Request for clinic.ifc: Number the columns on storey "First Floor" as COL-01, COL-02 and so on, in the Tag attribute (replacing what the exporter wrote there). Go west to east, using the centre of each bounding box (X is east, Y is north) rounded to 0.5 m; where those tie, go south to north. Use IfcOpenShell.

First a look at what the model holds.

```python
import ifcopenshell
import ifcopenshell.util.element
import ifcopenshell.util.placement

model = ifcopenshell.open("clinic.ifc")
print(model.schema)
storey = next(s for s in model.by_type("IfcBuildingStorey") if s.Name == "First Floor")
columns = [e for e in ifcopenshell.util.element.get_decomposition(storey) if e.is_a("IfcColumn")]
for e in sorted(columns, key=lambda e: e.id()):
    origin = ifcopenshell.util.placement.get_local_placement(e.ObjectPlacement)[:3, 3]
    print(e.id(), e.Tag, e.Name, origin.round(2) + 0.0, sep=" | ")
```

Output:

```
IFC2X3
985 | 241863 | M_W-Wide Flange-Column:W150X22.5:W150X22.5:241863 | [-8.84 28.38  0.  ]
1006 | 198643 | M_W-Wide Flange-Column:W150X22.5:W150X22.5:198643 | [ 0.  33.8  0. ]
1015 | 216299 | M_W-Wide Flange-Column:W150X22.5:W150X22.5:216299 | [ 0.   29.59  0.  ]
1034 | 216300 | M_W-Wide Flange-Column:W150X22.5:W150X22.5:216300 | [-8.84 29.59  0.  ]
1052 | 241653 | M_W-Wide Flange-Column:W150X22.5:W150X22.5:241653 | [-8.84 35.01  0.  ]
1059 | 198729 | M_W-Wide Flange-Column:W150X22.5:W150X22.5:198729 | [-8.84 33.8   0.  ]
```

```python
import ifcopenshell
import ifcopenshell.geom
import ifcopenshell.util.element
import ifcopenshell.util.shape

model = ifcopenshell.open("clinic.ifc")
settings = ifcopenshell.geom.settings()
settings.set("use-world-coords", True)


def centre(element):
    shape = ifcopenshell.geom.create_shape(settings, element)
    return ifcopenshell.util.shape.get_bbox_centroid(shape.geometry)


storey = next(s for s in model.by_type("IfcBuildingStorey") if s.Name == "First Floor")
columns = [e for e in ifcopenshell.util.element.get_decomposition(storey) if e.is_a("IfcColumn")]

# Insertion points can sit at a corner or the storey origin, so sort by the geometry (in metres).
centres = {e: centre(e) for e in columns}
columns.sort(key=lambda e: (round(centres[e][0] / 0.5), centres[e][1]))

for i, e in enumerate(columns, start=1):
    number = f"COL-{i:02d}"
    e.Tag = number
    print(e.id(), number)

model.write("clinic_edited.ifc")
```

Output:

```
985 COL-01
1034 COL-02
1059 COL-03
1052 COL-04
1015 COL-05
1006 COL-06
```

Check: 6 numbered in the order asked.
